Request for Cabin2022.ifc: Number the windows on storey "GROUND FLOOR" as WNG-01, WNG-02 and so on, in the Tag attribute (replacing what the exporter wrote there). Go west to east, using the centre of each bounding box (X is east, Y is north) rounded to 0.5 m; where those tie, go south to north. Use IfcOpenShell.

First a look at what the model holds.

```python
import ifcopenshell
import ifcopenshell.util.element
import ifcopenshell.util.placement

model = ifcopenshell.open("Cabin2022.ifc")
print(model.schema)
storey = next(s for s in model.by_type("IfcBuildingStorey") if s.Name == "GROUND FLOOR")
windows = [e for e in ifcopenshell.util.element.get_decomposition(storey) if e.is_a("IfcWindow")]
for e in sorted(windows, key=lambda e: e.id()):
    origin = ifcopenshell.util.placement.get_local_placement(e.ObjectPlacement)[:3, 3]
    print(e.id(), e.Tag, e.Name, origin.round(2) + 0.0, sep=" | ")
```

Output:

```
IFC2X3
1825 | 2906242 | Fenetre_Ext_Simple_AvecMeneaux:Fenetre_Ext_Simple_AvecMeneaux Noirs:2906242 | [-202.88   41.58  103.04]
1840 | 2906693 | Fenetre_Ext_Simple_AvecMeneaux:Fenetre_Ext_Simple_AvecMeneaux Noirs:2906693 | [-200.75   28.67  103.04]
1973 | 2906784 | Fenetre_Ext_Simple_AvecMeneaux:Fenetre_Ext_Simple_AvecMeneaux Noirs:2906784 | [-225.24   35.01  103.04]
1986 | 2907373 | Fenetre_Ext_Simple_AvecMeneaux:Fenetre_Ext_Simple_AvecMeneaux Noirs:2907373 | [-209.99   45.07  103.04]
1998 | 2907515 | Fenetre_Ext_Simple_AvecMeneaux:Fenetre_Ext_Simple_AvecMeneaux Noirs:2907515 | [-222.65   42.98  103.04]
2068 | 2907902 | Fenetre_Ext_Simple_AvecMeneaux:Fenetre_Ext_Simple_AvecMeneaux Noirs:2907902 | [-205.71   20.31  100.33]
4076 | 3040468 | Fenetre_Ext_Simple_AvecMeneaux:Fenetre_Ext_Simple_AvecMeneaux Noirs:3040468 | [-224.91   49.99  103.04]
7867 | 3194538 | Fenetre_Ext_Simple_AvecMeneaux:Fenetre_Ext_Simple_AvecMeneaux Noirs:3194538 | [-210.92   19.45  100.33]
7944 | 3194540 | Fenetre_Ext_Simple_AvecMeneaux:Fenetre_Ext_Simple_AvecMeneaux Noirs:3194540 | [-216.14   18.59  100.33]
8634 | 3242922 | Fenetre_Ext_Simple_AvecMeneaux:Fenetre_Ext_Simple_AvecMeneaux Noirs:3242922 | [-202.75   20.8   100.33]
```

```python
import ifcopenshell
import ifcopenshell.geom
import ifcopenshell.util.element
import ifcopenshell.util.shape

model = ifcopenshell.open("Cabin2022.ifc")
settings = ifcopenshell.geom.settings()
settings.set("use-world-coords", True)


def centre(element):
    shape = ifcopenshell.geom.create_shape(settings, element)
    return ifcopenshell.util.shape.get_bbox_centroid(shape.geometry)


storey = next(s for s in model.by_type("IfcBuildingStorey") if s.Name == "GROUND FLOOR")
windows = [e for e in ifcopenshell.util.element.get_decomposition(storey) if e.is_a("IfcWindow")]

# Insertion points can sit at a corner or the storey origin, so sort by the geometry (in metres).
centres = {e: centre(e) for e in windows}
windows.sort(key=lambda e: (round(centres[e][0] / 0.5), centres[e][1]))

for i, e in enumerate(windows, start=1):
    number = f"WNG-{i:02d}"
    e.Tag = number
    print(e.id(), number)

model.write("Cabin2022-out.ifc")
```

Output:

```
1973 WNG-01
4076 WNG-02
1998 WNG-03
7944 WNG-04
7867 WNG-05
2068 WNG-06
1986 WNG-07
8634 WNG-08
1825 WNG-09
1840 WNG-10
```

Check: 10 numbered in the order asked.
